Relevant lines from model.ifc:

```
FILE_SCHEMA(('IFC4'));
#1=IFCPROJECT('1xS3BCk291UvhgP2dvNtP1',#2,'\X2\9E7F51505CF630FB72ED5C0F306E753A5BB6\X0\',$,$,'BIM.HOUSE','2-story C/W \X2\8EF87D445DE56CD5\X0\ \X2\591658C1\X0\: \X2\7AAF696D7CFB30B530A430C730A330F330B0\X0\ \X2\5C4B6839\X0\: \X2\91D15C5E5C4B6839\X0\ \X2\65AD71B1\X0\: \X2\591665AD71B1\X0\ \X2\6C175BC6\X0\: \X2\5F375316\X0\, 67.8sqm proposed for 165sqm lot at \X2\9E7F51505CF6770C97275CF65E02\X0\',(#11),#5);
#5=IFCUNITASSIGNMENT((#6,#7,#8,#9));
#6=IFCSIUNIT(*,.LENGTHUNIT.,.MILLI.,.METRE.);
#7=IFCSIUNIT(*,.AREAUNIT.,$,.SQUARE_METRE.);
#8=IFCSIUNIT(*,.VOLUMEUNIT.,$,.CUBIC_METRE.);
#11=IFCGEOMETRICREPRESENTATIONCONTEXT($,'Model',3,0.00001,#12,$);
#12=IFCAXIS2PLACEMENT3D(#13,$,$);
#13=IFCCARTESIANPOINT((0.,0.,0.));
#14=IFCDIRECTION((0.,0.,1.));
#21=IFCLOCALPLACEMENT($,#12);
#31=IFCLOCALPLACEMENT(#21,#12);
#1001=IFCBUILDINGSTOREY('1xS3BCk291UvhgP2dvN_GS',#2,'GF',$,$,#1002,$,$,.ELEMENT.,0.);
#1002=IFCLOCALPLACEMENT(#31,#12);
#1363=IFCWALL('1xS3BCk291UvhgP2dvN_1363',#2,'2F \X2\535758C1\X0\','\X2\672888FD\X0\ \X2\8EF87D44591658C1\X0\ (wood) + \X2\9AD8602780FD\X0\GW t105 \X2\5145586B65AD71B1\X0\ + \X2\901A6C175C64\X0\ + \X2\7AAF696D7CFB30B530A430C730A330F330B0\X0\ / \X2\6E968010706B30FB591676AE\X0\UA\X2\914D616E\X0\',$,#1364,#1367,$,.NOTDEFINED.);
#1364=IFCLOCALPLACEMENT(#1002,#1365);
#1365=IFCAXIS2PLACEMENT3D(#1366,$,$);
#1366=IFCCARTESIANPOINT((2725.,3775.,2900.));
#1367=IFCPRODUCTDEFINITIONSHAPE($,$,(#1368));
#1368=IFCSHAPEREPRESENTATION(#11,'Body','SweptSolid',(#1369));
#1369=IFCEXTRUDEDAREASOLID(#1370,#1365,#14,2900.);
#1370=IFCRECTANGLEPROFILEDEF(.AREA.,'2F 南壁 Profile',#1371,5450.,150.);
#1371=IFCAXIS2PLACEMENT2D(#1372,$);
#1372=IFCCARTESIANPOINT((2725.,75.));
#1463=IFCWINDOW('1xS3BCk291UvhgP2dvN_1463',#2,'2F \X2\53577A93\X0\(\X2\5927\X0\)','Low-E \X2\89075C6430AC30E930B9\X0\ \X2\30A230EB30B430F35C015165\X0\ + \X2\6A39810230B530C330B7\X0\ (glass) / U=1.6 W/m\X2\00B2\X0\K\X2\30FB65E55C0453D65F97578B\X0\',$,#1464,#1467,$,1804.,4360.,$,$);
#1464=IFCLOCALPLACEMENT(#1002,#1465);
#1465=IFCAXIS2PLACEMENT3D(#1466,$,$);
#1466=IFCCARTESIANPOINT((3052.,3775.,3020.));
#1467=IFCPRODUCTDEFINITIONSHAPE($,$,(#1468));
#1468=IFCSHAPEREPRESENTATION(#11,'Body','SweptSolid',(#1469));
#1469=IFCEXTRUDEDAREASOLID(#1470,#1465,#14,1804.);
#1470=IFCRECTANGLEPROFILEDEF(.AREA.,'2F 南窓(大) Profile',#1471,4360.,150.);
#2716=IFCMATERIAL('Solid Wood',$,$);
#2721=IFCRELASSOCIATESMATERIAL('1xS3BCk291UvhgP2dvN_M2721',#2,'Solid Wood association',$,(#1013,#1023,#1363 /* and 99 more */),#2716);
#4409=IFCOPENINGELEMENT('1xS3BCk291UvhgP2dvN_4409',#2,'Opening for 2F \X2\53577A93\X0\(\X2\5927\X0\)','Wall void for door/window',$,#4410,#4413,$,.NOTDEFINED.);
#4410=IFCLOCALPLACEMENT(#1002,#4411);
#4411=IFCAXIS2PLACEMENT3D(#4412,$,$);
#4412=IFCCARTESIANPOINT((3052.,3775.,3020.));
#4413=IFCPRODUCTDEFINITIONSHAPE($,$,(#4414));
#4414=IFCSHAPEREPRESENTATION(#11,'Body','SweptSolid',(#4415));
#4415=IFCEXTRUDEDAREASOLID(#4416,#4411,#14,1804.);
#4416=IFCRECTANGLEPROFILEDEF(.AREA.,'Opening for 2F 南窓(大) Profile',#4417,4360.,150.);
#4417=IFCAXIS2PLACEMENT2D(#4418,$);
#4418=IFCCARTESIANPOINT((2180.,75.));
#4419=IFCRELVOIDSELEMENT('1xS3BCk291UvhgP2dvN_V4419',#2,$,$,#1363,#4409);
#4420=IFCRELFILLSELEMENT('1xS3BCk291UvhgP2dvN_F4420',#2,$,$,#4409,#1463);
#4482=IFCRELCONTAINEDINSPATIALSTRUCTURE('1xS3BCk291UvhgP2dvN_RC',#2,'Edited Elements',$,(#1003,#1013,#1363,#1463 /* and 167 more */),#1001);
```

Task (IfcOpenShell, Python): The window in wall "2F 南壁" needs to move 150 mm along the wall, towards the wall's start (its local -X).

```python
import ifcopenshell
import ifcopenshell.api.geometry
import ifcopenshell.util.placement
import ifcopenshell.util.unit

model = ifcopenshell.open("model.ifc")
unit_scale = ifcopenshell.util.unit.calculate_unit_scale(model)

window = model.by_id(1463)
opening = window.FillsVoids[0].RelatingOpeningElement
wall = opening.VoidsElements[0].RelatingBuildingElement

wall_matrix = ifcopenshell.util.placement.get_local_placement(wall.ObjectPlacement)
shift = wall_matrix[:3, 0] * -0.15 / unit_scale
before = ifcopenshell.util.placement.get_local_placement(window.ObjectPlacement)[:3, 3].copy()

# The window is not placed relative to its opening, so move both.
for product in (opening, window):
    matrix = ifcopenshell.util.placement.get_local_placement(product.ObjectPlacement)
    matrix[:3, 3] += shift
    ifcopenshell.api.geometry.edit_object_placement(model, product=product, matrix=matrix, is_si=False)

after = ifcopenshell.util.placement.get_local_placement(window.ObjectPlacement)[:3, 3]
print("window moved by", (after - before).round(3) + 0.0)

model.write("model_rev.ifc")
```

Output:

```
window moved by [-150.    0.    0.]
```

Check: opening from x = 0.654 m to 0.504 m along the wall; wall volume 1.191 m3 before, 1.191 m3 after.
